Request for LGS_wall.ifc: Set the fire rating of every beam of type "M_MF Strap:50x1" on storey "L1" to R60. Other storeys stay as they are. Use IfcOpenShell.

First a look at what the model holds.

```python
import ifcopenshell
import ifcopenshell.util.element

model = ifcopenshell.open("LGS_wall.ifc")
print(model.schema)
storey = next(s for s in model.by_type("IfcBuildingStorey") if s.Name == "L1")
beams = [e for e in ifcopenshell.util.element.get_decomposition(storey) if e.is_a("IfcBeam")]
seen = {}
for e in beams:
    element_type = ifcopenshell.util.element.get_type(e)
    key = (element_type.Name if element_type != e and element_type else None, ifcopenshell.util.element.get_pset(e, "Pset_BeamCommon", "FireRating"))
    seen[key] = seen.get(key, 0) + 1
for (name, value), count in sorted(seen.items(), key=str):
    print(count, "x", name, "|", value)
```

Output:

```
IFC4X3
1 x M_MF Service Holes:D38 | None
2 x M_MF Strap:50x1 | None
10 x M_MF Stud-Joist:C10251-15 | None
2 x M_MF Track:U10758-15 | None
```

```python
import ifcopenshell
import ifcopenshell.api.pset
import ifcopenshell.util.element

model = ifcopenshell.open("LGS_wall.ifc")

storey = next(s for s in model.by_type("IfcBuildingStorey") if s.Name == "L1")
beams = [e for e in ifcopenshell.util.element.get_decomposition(storey) if e.is_a("IfcBeam")]

count = 0
for e in beams:
    element_type = ifcopenshell.util.element.get_type(e)
    if element_type in (None, e) or element_type.Name != "M_MF Strap:50x1":
        continue
    # add_pset returns the element's existing set when there is one.
    pset = ifcopenshell.api.pset.add_pset(model, product=e, name="Pset_BeamCommon")
    ifcopenshell.api.pset.edit_pset(model, pset=pset, properties={"FireRating": "R60"})
    count += 1

print(count, "beams updated")

model.write("LGS_wall_v2.ifc")
```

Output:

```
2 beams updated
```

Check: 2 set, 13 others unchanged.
